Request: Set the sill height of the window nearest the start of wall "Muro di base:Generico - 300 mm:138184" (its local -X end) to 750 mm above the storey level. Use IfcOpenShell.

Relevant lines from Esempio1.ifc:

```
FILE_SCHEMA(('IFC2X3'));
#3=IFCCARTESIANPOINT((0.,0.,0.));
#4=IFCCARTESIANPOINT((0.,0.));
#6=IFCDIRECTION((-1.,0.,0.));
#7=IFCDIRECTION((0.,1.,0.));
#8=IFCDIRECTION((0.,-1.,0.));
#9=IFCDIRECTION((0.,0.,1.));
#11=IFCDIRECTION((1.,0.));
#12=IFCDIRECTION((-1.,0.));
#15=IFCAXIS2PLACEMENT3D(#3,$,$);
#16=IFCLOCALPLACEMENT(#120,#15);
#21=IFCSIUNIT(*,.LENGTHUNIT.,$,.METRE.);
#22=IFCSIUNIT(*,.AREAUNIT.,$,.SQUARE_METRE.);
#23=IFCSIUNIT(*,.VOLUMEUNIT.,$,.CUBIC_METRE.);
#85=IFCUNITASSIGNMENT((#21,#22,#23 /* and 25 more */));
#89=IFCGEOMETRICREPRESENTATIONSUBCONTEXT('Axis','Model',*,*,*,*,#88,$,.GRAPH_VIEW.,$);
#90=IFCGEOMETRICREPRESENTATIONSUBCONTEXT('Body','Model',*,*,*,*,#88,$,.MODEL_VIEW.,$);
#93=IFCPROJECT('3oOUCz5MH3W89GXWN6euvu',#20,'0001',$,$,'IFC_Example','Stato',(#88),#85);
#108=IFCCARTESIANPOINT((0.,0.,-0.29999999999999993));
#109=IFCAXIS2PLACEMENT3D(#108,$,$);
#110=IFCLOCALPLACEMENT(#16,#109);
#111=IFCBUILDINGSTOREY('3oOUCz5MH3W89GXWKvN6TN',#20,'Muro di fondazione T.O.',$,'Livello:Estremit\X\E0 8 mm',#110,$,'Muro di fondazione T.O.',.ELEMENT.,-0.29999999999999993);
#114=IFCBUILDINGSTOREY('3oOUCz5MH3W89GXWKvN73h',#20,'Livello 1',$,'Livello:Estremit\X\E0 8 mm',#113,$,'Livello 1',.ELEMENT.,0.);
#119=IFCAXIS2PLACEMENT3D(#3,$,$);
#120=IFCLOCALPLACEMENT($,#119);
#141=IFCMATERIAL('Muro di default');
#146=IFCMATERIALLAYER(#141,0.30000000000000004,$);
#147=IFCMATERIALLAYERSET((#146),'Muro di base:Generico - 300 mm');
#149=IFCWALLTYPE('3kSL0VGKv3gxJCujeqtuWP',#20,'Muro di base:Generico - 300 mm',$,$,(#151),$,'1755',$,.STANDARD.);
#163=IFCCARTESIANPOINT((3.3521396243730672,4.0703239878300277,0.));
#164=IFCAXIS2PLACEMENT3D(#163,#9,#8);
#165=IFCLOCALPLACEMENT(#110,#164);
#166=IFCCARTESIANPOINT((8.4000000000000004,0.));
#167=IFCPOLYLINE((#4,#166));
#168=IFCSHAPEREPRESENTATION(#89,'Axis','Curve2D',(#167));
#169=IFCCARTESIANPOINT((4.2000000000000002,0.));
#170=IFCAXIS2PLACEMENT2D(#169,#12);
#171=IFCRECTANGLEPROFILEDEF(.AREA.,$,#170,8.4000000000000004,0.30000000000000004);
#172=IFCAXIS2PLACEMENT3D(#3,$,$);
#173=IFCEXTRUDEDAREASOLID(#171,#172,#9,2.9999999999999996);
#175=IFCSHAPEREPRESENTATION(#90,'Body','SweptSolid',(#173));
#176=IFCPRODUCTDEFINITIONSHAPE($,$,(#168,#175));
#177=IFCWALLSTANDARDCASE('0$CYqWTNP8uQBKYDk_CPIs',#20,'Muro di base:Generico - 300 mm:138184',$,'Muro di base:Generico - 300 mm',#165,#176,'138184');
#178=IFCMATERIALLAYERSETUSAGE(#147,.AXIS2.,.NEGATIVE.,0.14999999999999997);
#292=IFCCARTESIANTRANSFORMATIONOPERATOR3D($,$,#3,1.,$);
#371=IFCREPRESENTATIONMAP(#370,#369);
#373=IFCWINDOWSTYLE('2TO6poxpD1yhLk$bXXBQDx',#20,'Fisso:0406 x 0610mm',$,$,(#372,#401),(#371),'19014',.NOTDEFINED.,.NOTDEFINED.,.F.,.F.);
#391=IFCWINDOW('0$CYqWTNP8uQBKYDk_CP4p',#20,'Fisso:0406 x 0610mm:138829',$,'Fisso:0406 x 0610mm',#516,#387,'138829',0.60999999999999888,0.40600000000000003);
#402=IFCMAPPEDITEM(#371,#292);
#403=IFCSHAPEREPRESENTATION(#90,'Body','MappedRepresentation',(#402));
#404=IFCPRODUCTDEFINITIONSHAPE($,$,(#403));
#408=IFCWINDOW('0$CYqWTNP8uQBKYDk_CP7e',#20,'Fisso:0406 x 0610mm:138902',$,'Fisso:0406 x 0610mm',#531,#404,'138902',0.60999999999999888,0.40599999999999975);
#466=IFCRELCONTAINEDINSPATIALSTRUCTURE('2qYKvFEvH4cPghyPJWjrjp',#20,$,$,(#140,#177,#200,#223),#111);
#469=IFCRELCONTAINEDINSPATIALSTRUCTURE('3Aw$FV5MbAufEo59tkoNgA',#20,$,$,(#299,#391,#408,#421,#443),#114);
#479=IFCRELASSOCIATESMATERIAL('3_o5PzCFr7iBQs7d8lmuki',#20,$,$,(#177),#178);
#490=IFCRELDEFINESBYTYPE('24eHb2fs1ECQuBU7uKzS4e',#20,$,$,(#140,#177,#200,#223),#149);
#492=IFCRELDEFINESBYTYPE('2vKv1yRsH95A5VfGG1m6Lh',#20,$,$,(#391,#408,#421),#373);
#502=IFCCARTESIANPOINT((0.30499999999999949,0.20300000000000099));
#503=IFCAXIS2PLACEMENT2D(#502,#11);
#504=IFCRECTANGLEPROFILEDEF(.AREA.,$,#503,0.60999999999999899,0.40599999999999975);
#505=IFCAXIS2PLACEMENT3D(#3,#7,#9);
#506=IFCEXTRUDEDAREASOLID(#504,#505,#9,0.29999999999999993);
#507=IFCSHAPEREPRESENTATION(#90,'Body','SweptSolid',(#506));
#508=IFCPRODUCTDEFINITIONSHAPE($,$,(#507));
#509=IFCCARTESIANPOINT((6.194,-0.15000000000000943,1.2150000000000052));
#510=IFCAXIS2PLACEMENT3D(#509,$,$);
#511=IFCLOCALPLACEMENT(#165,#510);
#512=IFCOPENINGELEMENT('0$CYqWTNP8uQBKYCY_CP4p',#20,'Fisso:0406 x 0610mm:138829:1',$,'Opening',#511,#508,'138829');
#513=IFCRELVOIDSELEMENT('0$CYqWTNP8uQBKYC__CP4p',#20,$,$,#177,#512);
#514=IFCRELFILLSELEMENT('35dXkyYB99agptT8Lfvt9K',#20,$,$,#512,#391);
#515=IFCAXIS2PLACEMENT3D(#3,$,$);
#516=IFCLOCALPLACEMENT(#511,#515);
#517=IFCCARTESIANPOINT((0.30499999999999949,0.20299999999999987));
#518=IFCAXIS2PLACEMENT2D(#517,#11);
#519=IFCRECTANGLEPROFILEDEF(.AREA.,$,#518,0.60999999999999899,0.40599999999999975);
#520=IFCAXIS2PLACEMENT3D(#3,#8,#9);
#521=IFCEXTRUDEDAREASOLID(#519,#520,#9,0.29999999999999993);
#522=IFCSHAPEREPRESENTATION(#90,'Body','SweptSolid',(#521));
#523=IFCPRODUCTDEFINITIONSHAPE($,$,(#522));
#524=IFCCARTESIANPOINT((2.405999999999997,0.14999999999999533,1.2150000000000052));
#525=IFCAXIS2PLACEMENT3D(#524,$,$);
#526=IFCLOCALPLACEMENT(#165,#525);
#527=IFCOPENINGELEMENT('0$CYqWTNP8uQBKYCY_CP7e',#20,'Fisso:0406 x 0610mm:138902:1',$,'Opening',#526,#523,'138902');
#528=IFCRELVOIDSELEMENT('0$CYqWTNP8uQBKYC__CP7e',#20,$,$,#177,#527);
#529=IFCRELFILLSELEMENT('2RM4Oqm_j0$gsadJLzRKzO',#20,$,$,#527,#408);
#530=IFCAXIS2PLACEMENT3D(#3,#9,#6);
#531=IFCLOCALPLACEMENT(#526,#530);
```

```python
import numpy as np
import ifcopenshell
import ifcopenshell.api.geometry
import ifcopenshell.geom
import ifcopenshell.util.element
import ifcopenshell.util.placement
import ifcopenshell.util.shape
import ifcopenshell.util.unit

model = ifcopenshell.open("Esempio1.ifc")
unit_scale = ifcopenshell.util.unit.calculate_unit_scale(model)

window = model.by_id(408)
opening = window.FillsVoids[0].RelatingOpeningElement
storey = ifcopenshell.util.element.get_container(window, ifc_class="IfcBuildingStorey")
level = ifcopenshell.util.placement.get_local_placement(storey.ObjectPlacement)[2, 3]

# The opening's origin need not be at the sill, so measure its lowest point.
shape = ifcopenshell.geom.create_shape(ifcopenshell.geom.settings(), opening)
bottom = ifcopenshell.util.shape.get_shape_bottom_elevation(shape, shape.geometry) / unit_scale
dz = level + 0.75 / unit_scale - bottom

shift = np.array([0.0, 0.0, dz])
# The window is placed relative to its opening, so it follows when the opening moves.
matrix = ifcopenshell.util.placement.get_local_placement(opening.ObjectPlacement)
matrix[:3, 3] += shift
ifcopenshell.api.geometry.edit_object_placement(
    model, product=opening, matrix=matrix, is_si=False, should_transform_children=True
)

print(f"moved by {dz * unit_scale:+.3f} m")

model.write("Esempio1_edited.ifc")
```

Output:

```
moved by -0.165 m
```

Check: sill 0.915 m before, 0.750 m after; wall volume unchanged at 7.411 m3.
